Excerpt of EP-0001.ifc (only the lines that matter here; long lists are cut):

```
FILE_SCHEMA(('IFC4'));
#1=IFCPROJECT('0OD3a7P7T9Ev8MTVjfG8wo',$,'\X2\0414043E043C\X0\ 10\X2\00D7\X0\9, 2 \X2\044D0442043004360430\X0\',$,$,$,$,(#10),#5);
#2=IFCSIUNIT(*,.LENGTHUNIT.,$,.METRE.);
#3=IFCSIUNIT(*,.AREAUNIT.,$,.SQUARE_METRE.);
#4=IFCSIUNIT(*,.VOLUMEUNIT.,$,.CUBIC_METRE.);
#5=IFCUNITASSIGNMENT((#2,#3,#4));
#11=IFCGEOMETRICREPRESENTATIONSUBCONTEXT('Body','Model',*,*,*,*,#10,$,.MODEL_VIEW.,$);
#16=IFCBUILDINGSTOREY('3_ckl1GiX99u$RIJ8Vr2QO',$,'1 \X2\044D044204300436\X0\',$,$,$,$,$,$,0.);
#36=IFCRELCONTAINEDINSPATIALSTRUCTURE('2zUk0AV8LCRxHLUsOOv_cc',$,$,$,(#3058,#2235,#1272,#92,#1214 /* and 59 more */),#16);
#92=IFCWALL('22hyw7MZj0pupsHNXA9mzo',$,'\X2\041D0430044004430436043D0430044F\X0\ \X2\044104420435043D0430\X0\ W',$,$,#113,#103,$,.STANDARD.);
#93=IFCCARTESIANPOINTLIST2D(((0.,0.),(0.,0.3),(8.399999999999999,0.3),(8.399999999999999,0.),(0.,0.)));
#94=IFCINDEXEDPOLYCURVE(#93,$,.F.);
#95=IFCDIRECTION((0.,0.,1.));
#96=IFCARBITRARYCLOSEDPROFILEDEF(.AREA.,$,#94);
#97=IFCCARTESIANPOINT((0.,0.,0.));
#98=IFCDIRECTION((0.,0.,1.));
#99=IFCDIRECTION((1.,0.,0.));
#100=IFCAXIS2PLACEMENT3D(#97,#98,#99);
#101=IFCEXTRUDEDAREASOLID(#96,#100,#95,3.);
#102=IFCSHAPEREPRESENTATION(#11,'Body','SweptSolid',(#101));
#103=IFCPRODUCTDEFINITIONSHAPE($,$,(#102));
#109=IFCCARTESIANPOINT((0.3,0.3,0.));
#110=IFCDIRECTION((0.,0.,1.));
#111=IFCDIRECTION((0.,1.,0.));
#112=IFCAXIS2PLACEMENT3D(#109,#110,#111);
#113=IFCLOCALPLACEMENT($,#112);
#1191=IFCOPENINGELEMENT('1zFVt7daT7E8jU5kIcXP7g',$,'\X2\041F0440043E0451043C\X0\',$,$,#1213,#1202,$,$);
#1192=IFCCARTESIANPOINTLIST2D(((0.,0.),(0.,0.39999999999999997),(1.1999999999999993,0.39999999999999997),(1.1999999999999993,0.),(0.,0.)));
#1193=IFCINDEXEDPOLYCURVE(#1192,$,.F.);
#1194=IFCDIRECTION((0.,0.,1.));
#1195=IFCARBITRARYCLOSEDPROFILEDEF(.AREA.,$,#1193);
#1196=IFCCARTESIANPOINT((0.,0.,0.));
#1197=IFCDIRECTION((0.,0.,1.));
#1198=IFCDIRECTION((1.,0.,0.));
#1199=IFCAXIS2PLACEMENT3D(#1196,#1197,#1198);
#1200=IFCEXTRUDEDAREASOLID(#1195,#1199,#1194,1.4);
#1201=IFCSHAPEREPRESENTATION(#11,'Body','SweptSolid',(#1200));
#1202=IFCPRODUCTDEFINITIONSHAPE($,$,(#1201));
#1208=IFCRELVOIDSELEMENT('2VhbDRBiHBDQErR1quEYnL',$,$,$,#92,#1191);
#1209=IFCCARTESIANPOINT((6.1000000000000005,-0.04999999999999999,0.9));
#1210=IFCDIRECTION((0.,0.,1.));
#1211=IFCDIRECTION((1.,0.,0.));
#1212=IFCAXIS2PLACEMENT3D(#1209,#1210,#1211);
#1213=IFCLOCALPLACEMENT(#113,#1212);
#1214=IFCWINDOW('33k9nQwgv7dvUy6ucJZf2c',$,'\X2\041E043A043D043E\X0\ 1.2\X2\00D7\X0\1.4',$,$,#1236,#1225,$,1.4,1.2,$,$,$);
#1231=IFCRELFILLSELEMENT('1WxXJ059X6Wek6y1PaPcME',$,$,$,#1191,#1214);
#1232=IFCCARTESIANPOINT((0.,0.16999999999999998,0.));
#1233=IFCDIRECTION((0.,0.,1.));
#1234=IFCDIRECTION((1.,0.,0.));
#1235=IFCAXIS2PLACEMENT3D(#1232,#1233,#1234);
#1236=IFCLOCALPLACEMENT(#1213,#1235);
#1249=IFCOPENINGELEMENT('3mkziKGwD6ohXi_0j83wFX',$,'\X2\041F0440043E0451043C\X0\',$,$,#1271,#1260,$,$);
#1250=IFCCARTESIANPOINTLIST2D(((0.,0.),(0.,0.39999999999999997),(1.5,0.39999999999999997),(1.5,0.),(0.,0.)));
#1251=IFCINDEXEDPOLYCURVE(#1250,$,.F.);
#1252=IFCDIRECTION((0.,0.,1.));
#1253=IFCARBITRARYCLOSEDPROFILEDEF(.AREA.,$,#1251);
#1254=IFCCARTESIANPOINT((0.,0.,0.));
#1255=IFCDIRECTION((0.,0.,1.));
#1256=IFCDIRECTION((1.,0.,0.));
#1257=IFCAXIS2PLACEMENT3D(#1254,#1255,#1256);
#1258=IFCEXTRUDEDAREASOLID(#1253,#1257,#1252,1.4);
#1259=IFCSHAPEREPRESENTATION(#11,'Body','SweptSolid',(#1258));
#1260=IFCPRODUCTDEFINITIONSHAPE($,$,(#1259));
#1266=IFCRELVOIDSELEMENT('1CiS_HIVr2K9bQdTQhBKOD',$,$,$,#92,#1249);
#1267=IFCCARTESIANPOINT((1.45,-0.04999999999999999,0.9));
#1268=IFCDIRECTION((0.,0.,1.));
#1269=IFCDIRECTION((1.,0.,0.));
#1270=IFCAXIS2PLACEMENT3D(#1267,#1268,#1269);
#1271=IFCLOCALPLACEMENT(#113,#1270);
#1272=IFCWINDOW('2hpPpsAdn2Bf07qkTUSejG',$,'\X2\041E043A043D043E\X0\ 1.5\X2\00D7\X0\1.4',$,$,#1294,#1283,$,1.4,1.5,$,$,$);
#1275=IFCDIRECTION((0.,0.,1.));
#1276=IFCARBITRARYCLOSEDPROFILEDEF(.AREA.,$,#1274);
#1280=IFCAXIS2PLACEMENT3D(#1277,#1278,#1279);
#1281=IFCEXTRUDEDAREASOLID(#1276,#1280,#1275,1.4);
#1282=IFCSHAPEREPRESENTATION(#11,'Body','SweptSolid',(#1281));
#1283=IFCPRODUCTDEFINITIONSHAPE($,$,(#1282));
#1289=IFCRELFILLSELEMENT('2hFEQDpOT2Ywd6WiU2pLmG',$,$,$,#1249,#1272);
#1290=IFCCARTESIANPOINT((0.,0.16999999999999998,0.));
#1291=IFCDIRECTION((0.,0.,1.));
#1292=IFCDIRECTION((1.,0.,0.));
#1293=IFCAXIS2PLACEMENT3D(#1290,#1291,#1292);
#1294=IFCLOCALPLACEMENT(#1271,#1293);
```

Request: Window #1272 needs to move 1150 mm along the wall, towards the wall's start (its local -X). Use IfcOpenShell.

```python
import ifcopenshell
import ifcopenshell.api.geometry
import ifcopenshell.util.placement

model = ifcopenshell.open("EP-0001.ifc")

window = model.by_guid("2hpPpsAdn2Bf07qkTUSejG")
opening = window.FillsVoids[0].RelatingOpeningElement
wall = opening.VoidsElements[0].RelatingBuildingElement

wall_matrix = ifcopenshell.util.placement.get_local_placement(wall.ObjectPlacement)
shift = wall_matrix[:3, 0] * -1.15
before = ifcopenshell.util.placement.get_local_placement(window.ObjectPlacement)[:3, 3].copy()

# The window is placed relative to its opening, so it follows when the opening moves.
matrix = ifcopenshell.util.placement.get_local_placement(opening.ObjectPlacement)
matrix[:3, 3] += shift
ifcopenshell.api.geometry.edit_object_placement(
    model, product=opening, matrix=matrix, is_si=False, should_transform_children=True
)

after = ifcopenshell.util.placement.get_local_placement(window.ObjectPlacement)[:3, 3]
print("window moved by", (after - before).round(3) + 0.0)

model.write("EP-0001_edited.ifc")
```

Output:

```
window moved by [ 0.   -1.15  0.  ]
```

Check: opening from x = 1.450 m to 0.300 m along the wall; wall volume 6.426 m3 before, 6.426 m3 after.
